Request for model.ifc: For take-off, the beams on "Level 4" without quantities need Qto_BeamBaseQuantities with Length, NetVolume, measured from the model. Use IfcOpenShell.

First a look at what the model holds.

```python
import ifcopenshell
import ifcopenshell.util.element
import ifcopenshell.util.unit

model = ifcopenshell.open("model.ifc")
print(model.schema)
for unit_type in ("LENGTHUNIT", "AREAUNIT", "VOLUMEUNIT"):
    print(unit_type, ifcopenshell.util.unit.calculate_unit_scale(model, unit_type))
storey = next(s for s in model.by_type("IfcBuildingStorey") if s.Name == "Level 4")
beams = [e for e in ifcopenshell.util.element.get_decomposition(storey) if e.is_a("IfcBeam")]
for e in sorted(beams, key=lambda e: e.id()):
    print(e.id(), e.is_a(), e.Name, list(ifcopenshell.util.element.get_psets(e, qtos_only=True)), sep=" | ")
```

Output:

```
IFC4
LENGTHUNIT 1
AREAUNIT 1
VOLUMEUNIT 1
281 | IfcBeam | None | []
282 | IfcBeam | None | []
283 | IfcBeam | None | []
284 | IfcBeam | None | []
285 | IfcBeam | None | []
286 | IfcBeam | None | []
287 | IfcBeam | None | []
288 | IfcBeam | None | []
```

```python
import ifcopenshell
import ifcopenshell.api.pset
import ifcopenshell.geom
import ifcopenshell.util.element
import ifcopenshell.util.shape
import ifcopenshell.util.unit

model = ifcopenshell.open("model.ifc")
unit_scale = ifcopenshell.util.unit.calculate_unit_scale(model)
volume_scale = ifcopenshell.util.unit.calculate_unit_scale(model, "VOLUMEUNIT")
settings = ifcopenshell.geom.settings()

storey = next(s for s in model.by_type("IfcBuildingStorey") if s.Name == "Level 4")
beams = [e for e in ifcopenshell.util.element.get_decomposition(storey) if e.is_a("IfcBeam")]

for e in sorted(beams, key=lambda e: e.id()):
    if ifcopenshell.util.element.get_psets(e, qtos_only=True, should_inherit=False):
        continue
    # Geometry comes back in metres, in the element's own axes.
    shape = ifcopenshell.geom.create_shape(settings, e)
    values = {
        "Length": ifcopenshell.util.shape.get_max_xyz(shape.geometry) / unit_scale,
        "NetVolume": ifcopenshell.util.shape.get_volume(shape.geometry) / volume_scale,
    }
    qto = ifcopenshell.api.pset.add_qto(model, product=e, name="Qto_BeamBaseQuantities")
    ifcopenshell.api.pset.edit_qto(model, qto=qto, properties=values)
    print(e.id(), {k: round(v, 3) for k, v in values.items()})

model.write("model_rev.ifc")
```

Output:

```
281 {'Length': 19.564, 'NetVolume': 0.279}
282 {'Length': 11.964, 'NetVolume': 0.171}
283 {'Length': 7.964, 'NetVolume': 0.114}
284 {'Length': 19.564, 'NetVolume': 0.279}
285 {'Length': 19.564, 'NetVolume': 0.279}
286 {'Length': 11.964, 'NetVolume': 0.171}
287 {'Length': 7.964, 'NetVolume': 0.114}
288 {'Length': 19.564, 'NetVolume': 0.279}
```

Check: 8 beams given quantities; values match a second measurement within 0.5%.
